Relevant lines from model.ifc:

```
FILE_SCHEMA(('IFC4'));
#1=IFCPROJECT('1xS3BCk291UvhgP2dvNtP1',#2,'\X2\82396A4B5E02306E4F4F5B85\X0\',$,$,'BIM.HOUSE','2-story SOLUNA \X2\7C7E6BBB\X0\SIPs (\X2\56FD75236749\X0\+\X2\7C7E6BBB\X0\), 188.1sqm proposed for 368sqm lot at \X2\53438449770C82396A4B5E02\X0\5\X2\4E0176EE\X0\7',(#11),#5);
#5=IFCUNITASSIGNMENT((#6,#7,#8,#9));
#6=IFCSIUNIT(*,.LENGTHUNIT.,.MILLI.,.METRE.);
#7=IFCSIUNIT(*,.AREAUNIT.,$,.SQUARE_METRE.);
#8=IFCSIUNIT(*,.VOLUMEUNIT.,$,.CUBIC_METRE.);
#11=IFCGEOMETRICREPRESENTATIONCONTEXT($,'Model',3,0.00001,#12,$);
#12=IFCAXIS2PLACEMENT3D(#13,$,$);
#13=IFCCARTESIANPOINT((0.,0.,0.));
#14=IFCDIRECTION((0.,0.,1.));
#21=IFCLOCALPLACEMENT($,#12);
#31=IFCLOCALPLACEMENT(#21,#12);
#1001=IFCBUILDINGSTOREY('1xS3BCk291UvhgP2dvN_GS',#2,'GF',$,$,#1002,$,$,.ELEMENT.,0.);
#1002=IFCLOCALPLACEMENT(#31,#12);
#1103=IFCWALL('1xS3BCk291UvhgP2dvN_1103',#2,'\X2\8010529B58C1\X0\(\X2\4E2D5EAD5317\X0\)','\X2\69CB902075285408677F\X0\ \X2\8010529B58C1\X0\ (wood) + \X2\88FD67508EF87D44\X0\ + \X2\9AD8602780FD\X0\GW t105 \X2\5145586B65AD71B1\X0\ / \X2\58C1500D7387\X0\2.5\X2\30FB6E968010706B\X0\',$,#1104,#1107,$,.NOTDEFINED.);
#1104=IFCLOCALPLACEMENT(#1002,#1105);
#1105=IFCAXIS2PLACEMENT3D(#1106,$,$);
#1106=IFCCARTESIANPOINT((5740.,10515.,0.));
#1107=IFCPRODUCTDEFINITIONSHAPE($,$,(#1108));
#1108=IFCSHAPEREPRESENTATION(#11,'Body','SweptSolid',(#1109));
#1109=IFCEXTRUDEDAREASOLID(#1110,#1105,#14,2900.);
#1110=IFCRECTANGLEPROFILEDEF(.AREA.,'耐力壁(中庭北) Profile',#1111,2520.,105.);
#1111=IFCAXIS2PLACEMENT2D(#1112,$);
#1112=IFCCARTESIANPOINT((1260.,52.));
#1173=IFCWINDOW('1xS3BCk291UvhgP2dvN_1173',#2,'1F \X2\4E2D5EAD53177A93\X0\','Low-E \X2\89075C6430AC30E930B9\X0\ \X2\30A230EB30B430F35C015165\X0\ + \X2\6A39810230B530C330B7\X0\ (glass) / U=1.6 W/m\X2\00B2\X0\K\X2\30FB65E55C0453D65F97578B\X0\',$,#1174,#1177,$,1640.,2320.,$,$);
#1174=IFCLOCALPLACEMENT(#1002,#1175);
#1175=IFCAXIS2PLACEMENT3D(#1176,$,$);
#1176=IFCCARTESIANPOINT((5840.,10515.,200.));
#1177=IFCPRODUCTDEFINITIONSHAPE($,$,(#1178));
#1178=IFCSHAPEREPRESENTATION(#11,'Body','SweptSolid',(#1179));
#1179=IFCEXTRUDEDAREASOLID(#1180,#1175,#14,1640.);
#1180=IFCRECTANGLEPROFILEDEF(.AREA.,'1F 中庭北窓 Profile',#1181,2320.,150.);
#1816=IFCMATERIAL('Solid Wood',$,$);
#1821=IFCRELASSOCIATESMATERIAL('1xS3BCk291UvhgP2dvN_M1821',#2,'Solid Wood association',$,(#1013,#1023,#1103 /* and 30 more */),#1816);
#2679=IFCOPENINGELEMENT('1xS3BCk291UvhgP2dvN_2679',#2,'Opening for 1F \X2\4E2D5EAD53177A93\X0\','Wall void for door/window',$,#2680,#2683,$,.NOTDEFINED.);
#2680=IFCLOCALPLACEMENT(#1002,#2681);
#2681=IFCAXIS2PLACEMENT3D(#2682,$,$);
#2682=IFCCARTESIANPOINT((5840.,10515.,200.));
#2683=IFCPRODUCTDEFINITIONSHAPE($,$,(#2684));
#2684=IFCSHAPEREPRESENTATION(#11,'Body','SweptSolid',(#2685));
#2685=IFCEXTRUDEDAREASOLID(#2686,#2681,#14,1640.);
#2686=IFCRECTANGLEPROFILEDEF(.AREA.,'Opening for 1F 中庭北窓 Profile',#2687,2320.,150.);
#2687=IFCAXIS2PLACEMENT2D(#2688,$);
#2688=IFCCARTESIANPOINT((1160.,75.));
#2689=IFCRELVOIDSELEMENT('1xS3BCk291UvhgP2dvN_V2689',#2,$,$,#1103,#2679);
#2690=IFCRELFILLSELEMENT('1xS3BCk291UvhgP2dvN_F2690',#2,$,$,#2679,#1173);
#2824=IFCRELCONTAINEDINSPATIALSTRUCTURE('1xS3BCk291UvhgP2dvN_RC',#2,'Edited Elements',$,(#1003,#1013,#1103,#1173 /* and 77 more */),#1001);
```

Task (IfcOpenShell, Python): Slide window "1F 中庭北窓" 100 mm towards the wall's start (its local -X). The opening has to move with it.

```python
import ifcopenshell
import ifcopenshell.api.geometry
import ifcopenshell.util.placement

model = ifcopenshell.open("model.ifc")

window = model.by_guid("1xS3BCk291UvhgP2dvN_1173")
opening = window.FillsVoids[0].RelatingOpeningElement
wall = opening.VoidsElements[0].RelatingBuildingElement

wall_matrix = ifcopenshell.util.placement.get_local_placement(wall.ObjectPlacement)
shift = wall_matrix[:3, 0] * -100.0
before = ifcopenshell.util.placement.get_local_placement(window.ObjectPlacement)[:3, 3].copy()

# The window is not placed relative to its opening, so move both.
for product in (opening, window):
    matrix = ifcopenshell.util.placement.get_local_placement(product.ObjectPlacement)
    matrix[:3, 3] += shift
    ifcopenshell.api.geometry.edit_object_placement(model, product=product, matrix=matrix, is_si=False)

after = ifcopenshell.util.placement.get_local_placement(window.ObjectPlacement)[:3, 3]
print("window moved by", (after - before).round(3) + 0.0)

model.write("model_edited.ifc")
```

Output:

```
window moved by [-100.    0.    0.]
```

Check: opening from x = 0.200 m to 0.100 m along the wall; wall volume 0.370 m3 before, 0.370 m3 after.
